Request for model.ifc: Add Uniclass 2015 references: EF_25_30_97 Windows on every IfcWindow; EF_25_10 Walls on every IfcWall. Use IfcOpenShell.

First a look at what the model holds.

```python
import ifcopenshell

model = ifcopenshell.open("model.ifc")
print(model.schema)
print("classifications:", [c.Name for c in model.by_type("IfcClassification")])
for ifc_class in ("IfcDoor", "IfcRoof", "IfcStair", "IfcWall", "IfcWindow"):
    print(ifc_class, len(model.by_type(ifc_class)))
```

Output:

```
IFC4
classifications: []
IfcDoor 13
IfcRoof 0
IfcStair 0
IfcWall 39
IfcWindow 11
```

```python
import ifcopenshell
import ifcopenshell.api.classification

model = ifcopenshell.open("model.ifc")

system = ifcopenshell.api.classification.add_classification(model, classification="Uniclass 2015")

codes = {
    "IfcWindow": ("EF_25_30_97", "Windows"),
    "IfcWall": ("EF_25_10", "Walls"),
}
for ifc_class, (code, name) in codes.items():
    products = model.by_type(ifc_class)
    ifcopenshell.api.classification.add_reference(
        model, products=products, classification=system, identification=code, name=name
    )
    print(code, len(products))

model.write("model_rev.ifc")
```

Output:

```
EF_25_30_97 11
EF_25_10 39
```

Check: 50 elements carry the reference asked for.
